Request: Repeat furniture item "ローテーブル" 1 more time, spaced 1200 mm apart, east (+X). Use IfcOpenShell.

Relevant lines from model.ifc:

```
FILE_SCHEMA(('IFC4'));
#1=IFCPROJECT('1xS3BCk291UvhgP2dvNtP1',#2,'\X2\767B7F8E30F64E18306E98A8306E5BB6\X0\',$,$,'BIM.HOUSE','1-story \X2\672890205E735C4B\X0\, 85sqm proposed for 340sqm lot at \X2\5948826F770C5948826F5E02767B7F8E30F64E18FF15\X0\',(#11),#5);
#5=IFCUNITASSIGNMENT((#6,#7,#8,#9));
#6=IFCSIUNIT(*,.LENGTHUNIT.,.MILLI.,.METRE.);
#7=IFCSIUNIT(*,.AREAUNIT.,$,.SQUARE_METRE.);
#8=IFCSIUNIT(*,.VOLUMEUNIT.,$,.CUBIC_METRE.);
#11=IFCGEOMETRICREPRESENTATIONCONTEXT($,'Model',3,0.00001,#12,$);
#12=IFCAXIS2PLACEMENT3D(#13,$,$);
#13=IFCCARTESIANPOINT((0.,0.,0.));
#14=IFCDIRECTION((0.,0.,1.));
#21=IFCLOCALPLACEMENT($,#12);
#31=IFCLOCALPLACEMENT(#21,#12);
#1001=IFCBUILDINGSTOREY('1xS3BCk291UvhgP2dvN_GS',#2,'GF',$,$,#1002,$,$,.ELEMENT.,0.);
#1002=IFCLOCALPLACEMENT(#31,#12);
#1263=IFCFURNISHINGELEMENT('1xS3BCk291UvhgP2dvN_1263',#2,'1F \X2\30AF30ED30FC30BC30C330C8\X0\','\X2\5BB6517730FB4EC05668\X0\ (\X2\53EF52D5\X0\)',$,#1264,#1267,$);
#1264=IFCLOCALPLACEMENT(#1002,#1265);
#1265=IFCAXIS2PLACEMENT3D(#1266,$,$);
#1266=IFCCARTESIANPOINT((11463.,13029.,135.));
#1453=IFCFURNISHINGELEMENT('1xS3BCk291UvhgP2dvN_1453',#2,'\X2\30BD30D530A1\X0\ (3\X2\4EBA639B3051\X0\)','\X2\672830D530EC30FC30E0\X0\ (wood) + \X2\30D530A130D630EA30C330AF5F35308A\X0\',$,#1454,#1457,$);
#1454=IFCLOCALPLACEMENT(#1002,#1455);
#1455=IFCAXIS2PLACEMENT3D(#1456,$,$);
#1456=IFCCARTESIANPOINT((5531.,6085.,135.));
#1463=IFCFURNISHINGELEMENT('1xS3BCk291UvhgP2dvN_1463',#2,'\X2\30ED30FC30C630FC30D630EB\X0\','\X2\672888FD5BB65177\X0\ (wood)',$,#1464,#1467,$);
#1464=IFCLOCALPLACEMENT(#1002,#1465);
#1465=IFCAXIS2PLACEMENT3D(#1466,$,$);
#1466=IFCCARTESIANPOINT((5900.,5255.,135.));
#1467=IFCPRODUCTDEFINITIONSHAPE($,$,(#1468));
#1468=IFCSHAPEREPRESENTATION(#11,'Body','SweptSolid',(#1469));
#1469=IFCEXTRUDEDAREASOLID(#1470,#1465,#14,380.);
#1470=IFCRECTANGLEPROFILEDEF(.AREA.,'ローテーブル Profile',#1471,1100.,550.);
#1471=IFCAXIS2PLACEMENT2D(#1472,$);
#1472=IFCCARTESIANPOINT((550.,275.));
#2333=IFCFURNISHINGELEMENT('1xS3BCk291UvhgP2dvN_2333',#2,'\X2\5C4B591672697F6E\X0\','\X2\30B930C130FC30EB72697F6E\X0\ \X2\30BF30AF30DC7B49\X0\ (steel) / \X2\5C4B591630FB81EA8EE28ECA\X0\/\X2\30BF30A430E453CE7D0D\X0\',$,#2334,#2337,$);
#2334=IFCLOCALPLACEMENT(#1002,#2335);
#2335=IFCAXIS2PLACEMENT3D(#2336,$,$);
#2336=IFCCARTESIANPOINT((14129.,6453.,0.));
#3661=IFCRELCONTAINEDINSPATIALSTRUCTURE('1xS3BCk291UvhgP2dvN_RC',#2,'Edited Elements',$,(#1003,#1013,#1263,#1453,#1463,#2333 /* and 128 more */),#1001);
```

```python
import numpy as np
import ifcopenshell
import ifcopenshell.api.geometry
import ifcopenshell.api.root
import ifcopenshell.util.element
import ifcopenshell.util.placement
import ifcopenshell.util.unit

model = ifcopenshell.open("model.ifc")
unit_scale = ifcopenshell.util.unit.calculate_unit_scale(model)


def reuse_history(source, copy):
    """copy_class also copies each property set's owner history, people and application; keep the originals."""
    for rel in copy.IsDefinedBy:
        if rel.is_a("IfcRelDefinesByProperties") and (history := rel.RelatingPropertyDefinition.OwnerHistory):
            rel.RelatingPropertyDefinition.OwnerHistory = source.OwnerHistory
            ifcopenshell.util.element.remove_deep2(model, history)


source = model.by_guid("1xS3BCk291UvhgP2dvN_1463")
base = ifcopenshell.util.placement.get_local_placement(source.ObjectPlacement)
step = np.array([1.0, 0.0, 0.0]) * 1.2 / unit_scale

for i in range(1, 2):
    copy = ifcopenshell.api.root.copy_class(model, product=source)
    copy.Representation = ifcopenshell.util.element.copy_deep(
        model, source.Representation, exclude=["IfcGeometricRepresentationContext", "IfcRepresentationMap"]
    )
    reuse_history(source, copy)
    matrix = base.copy()
    matrix[:3, 3] += i * step
    print("added at", matrix[:3, 3].round(3) + 0.0)
    ifcopenshell.api.geometry.edit_object_placement(model, product=copy, matrix=matrix, is_si=False)

model.write("model_rev.ifc")
```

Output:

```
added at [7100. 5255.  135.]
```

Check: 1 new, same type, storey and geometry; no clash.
